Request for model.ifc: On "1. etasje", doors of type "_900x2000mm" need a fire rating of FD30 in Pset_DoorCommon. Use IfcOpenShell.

First a look at what the model holds.

```python
import ifcopenshell
import ifcopenshell.util.element

model = ifcopenshell.open("model.ifc")
print(model.schema)
storey = next(s for s in model.by_type("IfcBuildingStorey") if s.Name == "1. etasje")
doors = [e for e in ifcopenshell.util.element.get_decomposition(storey) if e.is_a("IfcDoor")]
seen = {}
for e in doors:
    element_type = ifcopenshell.util.element.get_type(e)
    key = (element_type.Name if element_type != e and element_type else None, ifcopenshell.util.element.get_pset(e, "Pset_DoorCommon", "FireRating"))
    seen[key] = seen.get(key, 0) + 1
for (name, value), count in sorted(seen.items(), key=str):
    print(count, "x", name, "|", value)
```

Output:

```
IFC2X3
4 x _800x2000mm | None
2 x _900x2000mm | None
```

```python
import ifcopenshell
import ifcopenshell.api.pset
import ifcopenshell.util.element

model = ifcopenshell.open("model.ifc")

storey = next(s for s in model.by_type("IfcBuildingStorey") if s.Name == "1. etasje")
doors = [e for e in ifcopenshell.util.element.get_decomposition(storey) if e.is_a("IfcDoor")]

count = 0
for e in doors:
    element_type = ifcopenshell.util.element.get_type(e)
    if element_type in (None, e) or element_type.Name != "_900x2000mm":
        continue
    # add_pset returns the element's existing set when there is one.
    pset = ifcopenshell.api.pset.add_pset(model, product=e, name="Pset_DoorCommon")
    ifcopenshell.api.pset.edit_pset(model, pset=pset, properties={"FireRating": "FD30"})
    count += 1

print(count, "doors updated")

model.write("model_v2.ifc")
```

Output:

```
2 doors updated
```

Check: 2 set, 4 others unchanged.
